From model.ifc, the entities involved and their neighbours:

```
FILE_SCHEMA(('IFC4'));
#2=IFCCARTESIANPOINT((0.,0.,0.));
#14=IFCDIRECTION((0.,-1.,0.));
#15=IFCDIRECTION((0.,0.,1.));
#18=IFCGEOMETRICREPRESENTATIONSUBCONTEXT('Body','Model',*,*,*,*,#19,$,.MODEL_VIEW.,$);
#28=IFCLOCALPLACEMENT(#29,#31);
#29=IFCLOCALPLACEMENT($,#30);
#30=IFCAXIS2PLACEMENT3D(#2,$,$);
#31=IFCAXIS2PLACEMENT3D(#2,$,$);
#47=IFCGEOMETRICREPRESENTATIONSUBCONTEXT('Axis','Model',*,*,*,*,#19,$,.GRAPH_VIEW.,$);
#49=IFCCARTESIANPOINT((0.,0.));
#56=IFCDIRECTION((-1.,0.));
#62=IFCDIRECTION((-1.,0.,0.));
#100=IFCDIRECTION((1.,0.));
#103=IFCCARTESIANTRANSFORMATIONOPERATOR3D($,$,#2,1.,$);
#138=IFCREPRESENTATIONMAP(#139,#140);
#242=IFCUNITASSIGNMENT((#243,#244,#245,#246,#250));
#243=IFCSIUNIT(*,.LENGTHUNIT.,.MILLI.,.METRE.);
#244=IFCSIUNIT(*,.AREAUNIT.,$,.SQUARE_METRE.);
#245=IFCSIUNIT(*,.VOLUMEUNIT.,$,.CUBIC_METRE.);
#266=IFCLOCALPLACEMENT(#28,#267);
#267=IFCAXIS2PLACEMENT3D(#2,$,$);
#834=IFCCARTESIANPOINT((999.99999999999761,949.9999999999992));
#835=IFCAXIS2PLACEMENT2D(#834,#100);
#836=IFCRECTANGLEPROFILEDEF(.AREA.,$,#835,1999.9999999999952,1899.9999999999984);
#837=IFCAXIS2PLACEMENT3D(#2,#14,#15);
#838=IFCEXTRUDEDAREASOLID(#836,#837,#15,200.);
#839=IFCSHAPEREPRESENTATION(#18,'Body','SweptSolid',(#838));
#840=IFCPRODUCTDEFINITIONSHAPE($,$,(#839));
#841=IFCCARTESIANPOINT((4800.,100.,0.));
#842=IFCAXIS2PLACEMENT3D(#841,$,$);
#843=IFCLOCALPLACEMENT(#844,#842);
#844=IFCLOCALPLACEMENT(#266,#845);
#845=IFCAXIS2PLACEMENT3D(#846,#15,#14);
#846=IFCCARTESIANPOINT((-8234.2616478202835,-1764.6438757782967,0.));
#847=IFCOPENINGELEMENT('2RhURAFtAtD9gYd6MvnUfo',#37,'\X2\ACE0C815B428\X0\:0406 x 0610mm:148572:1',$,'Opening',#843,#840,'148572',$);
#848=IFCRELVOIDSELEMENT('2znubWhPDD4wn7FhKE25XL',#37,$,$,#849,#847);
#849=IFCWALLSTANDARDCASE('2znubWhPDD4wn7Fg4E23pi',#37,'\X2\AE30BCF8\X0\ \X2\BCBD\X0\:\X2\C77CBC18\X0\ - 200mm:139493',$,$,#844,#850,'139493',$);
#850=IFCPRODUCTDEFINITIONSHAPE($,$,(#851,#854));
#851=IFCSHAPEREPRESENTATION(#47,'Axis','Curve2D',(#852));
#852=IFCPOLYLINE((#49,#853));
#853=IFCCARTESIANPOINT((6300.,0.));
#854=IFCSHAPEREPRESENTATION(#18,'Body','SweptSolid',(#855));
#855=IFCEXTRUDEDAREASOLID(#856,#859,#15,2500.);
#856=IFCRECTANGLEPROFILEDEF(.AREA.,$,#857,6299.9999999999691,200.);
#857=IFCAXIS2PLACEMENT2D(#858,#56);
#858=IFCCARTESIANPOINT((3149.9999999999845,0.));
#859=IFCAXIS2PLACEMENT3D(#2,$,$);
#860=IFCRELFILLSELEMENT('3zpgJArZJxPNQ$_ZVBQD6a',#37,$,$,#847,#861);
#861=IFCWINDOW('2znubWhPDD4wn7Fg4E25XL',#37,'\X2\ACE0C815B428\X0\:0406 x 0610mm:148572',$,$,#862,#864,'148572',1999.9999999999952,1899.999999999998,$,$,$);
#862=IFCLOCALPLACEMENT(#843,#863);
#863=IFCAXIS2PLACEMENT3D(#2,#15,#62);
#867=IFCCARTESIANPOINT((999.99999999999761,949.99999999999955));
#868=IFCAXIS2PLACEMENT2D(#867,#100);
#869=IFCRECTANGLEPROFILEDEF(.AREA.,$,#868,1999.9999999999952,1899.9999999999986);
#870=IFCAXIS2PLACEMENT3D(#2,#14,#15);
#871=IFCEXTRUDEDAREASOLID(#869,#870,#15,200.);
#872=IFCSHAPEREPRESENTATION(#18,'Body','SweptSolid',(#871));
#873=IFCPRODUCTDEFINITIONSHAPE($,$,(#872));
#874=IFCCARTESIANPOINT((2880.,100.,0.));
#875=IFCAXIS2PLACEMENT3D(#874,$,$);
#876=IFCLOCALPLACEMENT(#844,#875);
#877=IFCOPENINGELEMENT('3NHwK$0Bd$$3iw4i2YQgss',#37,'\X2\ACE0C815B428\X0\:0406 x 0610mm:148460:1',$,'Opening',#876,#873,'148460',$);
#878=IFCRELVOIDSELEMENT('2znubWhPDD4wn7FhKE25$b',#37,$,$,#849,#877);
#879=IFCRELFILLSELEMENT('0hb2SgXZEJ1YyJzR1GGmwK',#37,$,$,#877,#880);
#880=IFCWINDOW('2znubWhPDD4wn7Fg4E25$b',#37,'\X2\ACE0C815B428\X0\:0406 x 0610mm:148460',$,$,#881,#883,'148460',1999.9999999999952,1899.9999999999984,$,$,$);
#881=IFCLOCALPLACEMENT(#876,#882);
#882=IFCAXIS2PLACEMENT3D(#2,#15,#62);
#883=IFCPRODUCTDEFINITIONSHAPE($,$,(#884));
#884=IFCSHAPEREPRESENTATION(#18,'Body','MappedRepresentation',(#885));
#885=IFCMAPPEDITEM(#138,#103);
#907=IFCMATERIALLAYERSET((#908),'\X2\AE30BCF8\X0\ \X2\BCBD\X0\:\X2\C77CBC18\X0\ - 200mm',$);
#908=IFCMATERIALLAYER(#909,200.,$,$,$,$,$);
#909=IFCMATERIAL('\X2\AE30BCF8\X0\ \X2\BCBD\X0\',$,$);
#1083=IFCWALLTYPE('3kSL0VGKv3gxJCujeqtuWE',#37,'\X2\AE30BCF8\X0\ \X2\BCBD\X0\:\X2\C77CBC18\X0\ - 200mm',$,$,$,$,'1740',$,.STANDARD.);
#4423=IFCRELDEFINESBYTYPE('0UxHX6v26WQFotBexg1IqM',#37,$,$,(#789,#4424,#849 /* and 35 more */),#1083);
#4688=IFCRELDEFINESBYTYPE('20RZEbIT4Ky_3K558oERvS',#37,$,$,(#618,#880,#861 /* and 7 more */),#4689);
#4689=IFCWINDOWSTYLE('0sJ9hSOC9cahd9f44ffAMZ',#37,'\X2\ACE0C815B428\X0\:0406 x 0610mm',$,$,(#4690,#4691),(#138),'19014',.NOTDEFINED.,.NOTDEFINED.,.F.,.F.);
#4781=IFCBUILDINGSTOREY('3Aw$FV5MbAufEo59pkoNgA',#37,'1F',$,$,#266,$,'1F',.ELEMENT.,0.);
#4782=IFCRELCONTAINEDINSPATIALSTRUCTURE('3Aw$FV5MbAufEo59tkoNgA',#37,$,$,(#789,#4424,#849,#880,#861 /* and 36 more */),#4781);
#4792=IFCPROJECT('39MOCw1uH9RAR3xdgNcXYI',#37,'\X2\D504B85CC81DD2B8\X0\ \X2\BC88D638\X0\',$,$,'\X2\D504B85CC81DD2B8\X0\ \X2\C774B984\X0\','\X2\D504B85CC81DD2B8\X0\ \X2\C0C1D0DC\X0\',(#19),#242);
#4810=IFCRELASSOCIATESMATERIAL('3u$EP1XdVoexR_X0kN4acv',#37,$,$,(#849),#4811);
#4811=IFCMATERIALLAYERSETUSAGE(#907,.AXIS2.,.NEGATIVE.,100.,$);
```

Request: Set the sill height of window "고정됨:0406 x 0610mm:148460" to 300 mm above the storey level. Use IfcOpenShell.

```python
import numpy as np
import ifcopenshell
import ifcopenshell.api.geometry
import ifcopenshell.geom
import ifcopenshell.util.element
import ifcopenshell.util.placement
import ifcopenshell.util.shape
import ifcopenshell.util.unit

model = ifcopenshell.open("model.ifc")
unit_scale = ifcopenshell.util.unit.calculate_unit_scale(model)

window = model.by_guid("2znubWhPDD4wn7Fg4E25$b")
opening = window.FillsVoids[0].RelatingOpeningElement
storey = ifcopenshell.util.element.get_container(window, ifc_class="IfcBuildingStorey")
level = ifcopenshell.util.placement.get_local_placement(storey.ObjectPlacement)[2, 3]

# The opening's origin need not be at the sill, so measure its lowest point.
shape = ifcopenshell.geom.create_shape(ifcopenshell.geom.settings(), opening)
bottom = ifcopenshell.util.shape.get_shape_bottom_elevation(shape, shape.geometry) / unit_scale
dz = level + 0.3 / unit_scale - bottom

shift = np.array([0.0, 0.0, dz])
# The window is placed relative to its opening, so it follows when the opening moves.
matrix = ifcopenshell.util.placement.get_local_placement(opening.ObjectPlacement)
matrix[:3, 3] += shift
ifcopenshell.api.geometry.edit_object_placement(
    model, product=opening, matrix=matrix, is_si=False, should_transform_children=True
)

print(f"moved by {dz * unit_scale:+.3f} m")

model.write("model_v2.ifc")
```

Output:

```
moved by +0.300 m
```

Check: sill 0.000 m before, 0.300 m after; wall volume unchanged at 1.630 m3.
